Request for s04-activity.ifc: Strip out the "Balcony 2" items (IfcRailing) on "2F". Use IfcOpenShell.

First a look at what the model holds.

```python
import ifcopenshell
import ifcopenshell.util.element

model = ifcopenshell.open("s04-activity.ifc")
print(model.schema)
storey = next(s for s in model.by_type("IfcBuildingStorey") if s.Name == "2F")
railings = [e for e in ifcopenshell.util.element.get_decomposition(storey) if e.is_a("IfcRailing")]
seen = {}
for e in railings:
    element_type = ifcopenshell.util.element.get_type(e)
    name = element_type.Name if element_type not in (None, e) else None
    seen[name] = seen.get(name, 0) + 1
for name, count in sorted(seen.items(), key=str):
    print(count, "x", name)
```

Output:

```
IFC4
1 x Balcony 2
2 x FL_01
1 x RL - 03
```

```python
import ifcopenshell
import ifcopenshell.api.root
import ifcopenshell.util.element

model = ifcopenshell.open("s04-activity.ifc")

storey = next(s for s in model.by_type("IfcBuildingStorey") if s.Name == "2F")
railings = [e for e in ifcopenshell.util.element.get_decomposition(storey) if e.is_a("IfcRailing")]
targets = [e for e in railings if (t := ifcopenshell.util.element.get_type(e)) not in (None, e) and t.Name == "Balcony 2"]

for e in targets:
    ifcopenshell.api.root.remove_product(model, product=e)
print(len(targets), "removed")

model.write("s04-activity-out.ifc")
```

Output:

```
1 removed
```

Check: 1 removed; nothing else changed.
